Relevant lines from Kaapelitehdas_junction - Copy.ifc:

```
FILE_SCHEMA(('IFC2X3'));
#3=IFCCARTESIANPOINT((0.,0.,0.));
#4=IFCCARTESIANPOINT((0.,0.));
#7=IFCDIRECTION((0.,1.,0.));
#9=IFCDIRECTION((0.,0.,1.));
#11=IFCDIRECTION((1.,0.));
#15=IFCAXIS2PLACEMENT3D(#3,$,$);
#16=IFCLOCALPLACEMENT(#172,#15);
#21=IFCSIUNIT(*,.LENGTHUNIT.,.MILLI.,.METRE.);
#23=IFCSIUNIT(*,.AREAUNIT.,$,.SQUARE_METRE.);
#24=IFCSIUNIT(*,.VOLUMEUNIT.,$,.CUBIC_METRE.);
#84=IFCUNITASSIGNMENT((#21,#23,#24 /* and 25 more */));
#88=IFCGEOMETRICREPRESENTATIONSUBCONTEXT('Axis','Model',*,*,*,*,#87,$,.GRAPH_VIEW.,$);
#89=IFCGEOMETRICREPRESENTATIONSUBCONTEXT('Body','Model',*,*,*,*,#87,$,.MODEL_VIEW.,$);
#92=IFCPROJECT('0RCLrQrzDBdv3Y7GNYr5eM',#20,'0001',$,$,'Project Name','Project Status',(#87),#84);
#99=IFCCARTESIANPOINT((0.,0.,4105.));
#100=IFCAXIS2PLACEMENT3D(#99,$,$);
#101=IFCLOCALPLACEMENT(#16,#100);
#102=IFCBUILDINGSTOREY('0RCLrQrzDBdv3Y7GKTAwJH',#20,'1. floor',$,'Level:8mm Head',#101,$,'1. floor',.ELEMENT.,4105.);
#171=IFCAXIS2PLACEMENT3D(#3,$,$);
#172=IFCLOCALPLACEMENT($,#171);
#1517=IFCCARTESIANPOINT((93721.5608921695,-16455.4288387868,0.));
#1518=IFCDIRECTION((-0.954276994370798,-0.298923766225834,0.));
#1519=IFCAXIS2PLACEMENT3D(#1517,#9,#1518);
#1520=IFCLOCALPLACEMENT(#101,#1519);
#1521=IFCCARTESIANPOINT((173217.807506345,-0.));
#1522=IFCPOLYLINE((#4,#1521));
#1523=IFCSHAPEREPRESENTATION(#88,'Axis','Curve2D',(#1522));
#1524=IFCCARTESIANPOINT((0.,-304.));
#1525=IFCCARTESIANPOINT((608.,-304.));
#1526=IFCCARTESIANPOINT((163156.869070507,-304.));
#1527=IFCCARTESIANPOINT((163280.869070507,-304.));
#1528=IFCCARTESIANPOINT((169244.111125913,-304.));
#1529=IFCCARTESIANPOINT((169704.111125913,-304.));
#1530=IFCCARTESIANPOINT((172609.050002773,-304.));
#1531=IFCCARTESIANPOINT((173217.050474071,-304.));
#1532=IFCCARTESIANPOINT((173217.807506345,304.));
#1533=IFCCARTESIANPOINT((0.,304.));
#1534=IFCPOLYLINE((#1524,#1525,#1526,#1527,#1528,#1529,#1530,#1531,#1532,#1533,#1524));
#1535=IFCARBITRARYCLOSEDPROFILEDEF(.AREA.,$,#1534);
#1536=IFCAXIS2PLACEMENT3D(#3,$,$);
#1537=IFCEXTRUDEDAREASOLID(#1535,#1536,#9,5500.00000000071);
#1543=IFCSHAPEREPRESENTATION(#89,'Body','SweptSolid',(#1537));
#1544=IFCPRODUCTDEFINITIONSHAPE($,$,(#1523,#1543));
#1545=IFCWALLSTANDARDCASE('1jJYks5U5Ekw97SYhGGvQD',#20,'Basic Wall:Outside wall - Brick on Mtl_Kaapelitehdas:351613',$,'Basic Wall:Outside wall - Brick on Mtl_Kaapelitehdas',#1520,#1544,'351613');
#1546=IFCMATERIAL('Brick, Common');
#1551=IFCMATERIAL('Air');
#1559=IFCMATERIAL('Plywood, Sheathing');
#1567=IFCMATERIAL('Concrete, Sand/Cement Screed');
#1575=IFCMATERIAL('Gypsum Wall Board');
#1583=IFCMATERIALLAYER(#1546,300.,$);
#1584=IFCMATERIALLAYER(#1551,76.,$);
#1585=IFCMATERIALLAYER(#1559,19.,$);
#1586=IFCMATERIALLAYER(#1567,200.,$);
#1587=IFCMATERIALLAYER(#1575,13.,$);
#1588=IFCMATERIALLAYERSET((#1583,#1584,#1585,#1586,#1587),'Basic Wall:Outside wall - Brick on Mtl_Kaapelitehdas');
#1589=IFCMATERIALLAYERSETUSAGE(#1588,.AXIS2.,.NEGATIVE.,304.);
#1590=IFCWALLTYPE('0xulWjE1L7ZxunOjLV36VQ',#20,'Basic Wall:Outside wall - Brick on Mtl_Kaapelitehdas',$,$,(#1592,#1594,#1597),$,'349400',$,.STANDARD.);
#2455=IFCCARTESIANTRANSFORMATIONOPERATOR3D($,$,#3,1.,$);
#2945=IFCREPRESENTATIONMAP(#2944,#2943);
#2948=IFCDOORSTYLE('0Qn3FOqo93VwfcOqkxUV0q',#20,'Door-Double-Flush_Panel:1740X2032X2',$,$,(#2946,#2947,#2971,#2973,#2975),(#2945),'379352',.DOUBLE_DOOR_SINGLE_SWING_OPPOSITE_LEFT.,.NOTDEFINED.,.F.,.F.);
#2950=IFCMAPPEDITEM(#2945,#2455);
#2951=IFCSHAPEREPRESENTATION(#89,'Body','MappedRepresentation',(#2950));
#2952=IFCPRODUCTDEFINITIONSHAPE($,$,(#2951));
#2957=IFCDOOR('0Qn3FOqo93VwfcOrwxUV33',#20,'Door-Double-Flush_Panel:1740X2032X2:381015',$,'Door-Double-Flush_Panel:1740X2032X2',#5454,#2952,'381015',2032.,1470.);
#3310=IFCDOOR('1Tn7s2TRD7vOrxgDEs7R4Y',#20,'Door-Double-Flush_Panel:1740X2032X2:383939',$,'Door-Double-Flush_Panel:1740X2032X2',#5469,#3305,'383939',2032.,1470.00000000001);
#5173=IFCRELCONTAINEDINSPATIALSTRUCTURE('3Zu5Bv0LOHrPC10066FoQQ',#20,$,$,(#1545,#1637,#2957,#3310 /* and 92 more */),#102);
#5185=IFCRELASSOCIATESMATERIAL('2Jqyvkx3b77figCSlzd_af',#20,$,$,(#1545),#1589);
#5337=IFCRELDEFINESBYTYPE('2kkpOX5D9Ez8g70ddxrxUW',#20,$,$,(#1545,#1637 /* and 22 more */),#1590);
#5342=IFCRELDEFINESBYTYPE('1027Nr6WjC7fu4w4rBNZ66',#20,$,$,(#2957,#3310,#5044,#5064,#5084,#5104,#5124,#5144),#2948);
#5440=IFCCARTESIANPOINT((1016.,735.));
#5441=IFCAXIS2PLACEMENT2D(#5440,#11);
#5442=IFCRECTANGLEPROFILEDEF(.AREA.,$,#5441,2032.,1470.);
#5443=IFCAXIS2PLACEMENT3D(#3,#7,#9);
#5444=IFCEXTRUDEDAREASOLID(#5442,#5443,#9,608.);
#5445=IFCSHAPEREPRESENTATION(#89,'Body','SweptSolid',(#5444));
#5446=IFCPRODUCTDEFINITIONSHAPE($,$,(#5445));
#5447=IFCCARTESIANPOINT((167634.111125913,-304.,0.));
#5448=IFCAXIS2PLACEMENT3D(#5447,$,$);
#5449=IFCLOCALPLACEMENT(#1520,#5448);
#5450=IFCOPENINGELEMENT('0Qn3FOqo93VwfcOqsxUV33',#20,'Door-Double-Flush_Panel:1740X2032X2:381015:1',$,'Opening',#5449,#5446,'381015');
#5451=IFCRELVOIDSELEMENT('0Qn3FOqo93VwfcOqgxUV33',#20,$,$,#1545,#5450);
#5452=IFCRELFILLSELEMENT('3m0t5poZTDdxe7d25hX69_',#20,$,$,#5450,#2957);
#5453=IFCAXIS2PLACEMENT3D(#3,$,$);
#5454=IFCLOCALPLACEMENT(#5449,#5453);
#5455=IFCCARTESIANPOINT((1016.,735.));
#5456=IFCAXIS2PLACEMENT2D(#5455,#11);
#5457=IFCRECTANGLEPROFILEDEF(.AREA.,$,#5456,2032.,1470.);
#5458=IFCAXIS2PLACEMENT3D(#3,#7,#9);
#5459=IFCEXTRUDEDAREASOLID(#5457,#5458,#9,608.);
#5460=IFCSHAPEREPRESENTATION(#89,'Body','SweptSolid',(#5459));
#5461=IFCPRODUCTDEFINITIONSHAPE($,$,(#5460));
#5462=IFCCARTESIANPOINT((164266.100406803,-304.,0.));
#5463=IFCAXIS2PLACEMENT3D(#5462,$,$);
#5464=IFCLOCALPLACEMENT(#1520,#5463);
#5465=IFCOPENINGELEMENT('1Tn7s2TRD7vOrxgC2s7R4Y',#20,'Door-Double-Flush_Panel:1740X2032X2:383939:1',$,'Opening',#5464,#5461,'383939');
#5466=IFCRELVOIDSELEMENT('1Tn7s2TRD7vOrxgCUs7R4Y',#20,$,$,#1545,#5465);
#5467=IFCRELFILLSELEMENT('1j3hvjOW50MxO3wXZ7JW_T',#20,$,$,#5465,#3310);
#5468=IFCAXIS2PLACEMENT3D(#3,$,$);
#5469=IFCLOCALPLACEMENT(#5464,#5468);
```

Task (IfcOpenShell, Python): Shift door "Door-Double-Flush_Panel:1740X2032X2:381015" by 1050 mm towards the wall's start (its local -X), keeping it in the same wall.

```python
import ifcopenshell
import ifcopenshell.api.geometry
import ifcopenshell.util.placement

model = ifcopenshell.open("Kaapelitehdas_junction - Copy.ifc")

door = model.by_guid("0Qn3FOqo93VwfcOrwxUV33")
opening = door.FillsVoids[0].RelatingOpeningElement
wall = opening.VoidsElements[0].RelatingBuildingElement

wall_matrix = ifcopenshell.util.placement.get_local_placement(wall.ObjectPlacement)
shift = wall_matrix[:3, 0] * -1050.0
before = ifcopenshell.util.placement.get_local_placement(door.ObjectPlacement)[:3, 3].copy()

# The door is placed relative to its opening, so it follows when the opening moves.
matrix = ifcopenshell.util.placement.get_local_placement(opening.ObjectPlacement)
matrix[:3, 3] += shift
ifcopenshell.api.geometry.edit_object_placement(
    model, product=opening, matrix=matrix, is_si=False, should_transform_children=True
)

after = ifcopenshell.util.placement.get_local_placement(door.ObjectPlacement)[:3, 3]
print("door moved by", (after - before).round(3) + 0.0)

model.write("Kaapelitehdas_junction - Copy_rev.ifc")
```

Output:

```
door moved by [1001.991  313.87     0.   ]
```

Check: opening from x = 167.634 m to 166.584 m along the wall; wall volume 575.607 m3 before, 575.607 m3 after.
